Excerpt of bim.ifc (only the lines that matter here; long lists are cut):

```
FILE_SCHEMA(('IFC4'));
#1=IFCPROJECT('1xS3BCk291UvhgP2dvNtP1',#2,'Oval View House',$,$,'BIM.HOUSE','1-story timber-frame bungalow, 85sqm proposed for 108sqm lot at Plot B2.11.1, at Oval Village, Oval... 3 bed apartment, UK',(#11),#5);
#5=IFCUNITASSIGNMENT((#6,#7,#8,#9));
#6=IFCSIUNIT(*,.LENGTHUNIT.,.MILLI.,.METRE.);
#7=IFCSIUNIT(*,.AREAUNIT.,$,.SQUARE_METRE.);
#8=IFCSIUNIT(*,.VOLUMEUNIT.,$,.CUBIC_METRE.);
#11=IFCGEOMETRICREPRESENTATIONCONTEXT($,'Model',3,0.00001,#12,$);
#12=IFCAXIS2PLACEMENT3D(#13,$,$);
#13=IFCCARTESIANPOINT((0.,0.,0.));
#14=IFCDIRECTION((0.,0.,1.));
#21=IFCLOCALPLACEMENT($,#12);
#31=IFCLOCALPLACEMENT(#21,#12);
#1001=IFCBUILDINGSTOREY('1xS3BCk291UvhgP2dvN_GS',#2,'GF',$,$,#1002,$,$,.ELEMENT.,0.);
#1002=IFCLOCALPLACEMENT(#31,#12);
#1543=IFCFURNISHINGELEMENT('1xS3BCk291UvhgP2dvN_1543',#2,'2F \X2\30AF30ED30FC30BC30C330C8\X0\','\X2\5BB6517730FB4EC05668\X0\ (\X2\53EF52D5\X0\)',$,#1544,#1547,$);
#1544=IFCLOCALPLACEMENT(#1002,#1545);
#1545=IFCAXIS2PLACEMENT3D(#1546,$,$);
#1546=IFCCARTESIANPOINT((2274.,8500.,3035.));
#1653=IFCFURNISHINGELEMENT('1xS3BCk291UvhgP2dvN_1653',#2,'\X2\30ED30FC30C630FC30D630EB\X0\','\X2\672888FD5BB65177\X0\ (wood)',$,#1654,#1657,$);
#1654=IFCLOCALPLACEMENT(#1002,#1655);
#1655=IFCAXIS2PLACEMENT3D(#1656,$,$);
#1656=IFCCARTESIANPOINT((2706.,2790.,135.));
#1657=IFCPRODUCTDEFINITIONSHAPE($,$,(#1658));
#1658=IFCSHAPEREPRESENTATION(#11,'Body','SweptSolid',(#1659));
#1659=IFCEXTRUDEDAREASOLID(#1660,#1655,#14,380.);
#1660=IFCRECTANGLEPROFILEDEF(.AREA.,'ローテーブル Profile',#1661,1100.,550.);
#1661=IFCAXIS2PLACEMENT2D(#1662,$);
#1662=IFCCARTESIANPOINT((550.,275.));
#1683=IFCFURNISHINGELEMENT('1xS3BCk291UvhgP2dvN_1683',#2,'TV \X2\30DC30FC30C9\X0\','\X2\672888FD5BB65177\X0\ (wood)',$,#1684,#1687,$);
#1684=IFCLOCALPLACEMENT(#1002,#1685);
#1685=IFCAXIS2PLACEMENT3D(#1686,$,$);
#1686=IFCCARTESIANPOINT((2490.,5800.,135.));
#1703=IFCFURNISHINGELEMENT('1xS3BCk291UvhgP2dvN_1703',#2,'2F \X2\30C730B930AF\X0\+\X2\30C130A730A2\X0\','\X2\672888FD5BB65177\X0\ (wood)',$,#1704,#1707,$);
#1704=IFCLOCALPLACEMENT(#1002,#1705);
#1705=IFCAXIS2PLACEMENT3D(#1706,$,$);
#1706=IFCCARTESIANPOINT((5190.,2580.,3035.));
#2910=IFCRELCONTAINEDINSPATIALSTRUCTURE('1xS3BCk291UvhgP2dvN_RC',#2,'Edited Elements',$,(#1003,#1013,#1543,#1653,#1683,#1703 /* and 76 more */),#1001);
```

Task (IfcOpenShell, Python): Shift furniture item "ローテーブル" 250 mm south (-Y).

```python
import ifcopenshell
import ifcopenshell.api.geometry
import ifcopenshell.util.placement
import ifcopenshell.util.unit

model = ifcopenshell.open("bim.ifc")
unit_scale = ifcopenshell.util.unit.calculate_unit_scale(model)

item = model.by_id(1653)
matrix = ifcopenshell.util.placement.get_local_placement(item.ObjectPlacement)
matrix[1, 3] -= 0.25 / unit_scale
ifcopenshell.api.geometry.edit_object_placement(model, product=item, matrix=matrix, is_si=False)

print(ifcopenshell.util.placement.get_local_placement(item.ObjectPlacement).round(3) + 0.0)

model.write("bim_updated.ifc")
```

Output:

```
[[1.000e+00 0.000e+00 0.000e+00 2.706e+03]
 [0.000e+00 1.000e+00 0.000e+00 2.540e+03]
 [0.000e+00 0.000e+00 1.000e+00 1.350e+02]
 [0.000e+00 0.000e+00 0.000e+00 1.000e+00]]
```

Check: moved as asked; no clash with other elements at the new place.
